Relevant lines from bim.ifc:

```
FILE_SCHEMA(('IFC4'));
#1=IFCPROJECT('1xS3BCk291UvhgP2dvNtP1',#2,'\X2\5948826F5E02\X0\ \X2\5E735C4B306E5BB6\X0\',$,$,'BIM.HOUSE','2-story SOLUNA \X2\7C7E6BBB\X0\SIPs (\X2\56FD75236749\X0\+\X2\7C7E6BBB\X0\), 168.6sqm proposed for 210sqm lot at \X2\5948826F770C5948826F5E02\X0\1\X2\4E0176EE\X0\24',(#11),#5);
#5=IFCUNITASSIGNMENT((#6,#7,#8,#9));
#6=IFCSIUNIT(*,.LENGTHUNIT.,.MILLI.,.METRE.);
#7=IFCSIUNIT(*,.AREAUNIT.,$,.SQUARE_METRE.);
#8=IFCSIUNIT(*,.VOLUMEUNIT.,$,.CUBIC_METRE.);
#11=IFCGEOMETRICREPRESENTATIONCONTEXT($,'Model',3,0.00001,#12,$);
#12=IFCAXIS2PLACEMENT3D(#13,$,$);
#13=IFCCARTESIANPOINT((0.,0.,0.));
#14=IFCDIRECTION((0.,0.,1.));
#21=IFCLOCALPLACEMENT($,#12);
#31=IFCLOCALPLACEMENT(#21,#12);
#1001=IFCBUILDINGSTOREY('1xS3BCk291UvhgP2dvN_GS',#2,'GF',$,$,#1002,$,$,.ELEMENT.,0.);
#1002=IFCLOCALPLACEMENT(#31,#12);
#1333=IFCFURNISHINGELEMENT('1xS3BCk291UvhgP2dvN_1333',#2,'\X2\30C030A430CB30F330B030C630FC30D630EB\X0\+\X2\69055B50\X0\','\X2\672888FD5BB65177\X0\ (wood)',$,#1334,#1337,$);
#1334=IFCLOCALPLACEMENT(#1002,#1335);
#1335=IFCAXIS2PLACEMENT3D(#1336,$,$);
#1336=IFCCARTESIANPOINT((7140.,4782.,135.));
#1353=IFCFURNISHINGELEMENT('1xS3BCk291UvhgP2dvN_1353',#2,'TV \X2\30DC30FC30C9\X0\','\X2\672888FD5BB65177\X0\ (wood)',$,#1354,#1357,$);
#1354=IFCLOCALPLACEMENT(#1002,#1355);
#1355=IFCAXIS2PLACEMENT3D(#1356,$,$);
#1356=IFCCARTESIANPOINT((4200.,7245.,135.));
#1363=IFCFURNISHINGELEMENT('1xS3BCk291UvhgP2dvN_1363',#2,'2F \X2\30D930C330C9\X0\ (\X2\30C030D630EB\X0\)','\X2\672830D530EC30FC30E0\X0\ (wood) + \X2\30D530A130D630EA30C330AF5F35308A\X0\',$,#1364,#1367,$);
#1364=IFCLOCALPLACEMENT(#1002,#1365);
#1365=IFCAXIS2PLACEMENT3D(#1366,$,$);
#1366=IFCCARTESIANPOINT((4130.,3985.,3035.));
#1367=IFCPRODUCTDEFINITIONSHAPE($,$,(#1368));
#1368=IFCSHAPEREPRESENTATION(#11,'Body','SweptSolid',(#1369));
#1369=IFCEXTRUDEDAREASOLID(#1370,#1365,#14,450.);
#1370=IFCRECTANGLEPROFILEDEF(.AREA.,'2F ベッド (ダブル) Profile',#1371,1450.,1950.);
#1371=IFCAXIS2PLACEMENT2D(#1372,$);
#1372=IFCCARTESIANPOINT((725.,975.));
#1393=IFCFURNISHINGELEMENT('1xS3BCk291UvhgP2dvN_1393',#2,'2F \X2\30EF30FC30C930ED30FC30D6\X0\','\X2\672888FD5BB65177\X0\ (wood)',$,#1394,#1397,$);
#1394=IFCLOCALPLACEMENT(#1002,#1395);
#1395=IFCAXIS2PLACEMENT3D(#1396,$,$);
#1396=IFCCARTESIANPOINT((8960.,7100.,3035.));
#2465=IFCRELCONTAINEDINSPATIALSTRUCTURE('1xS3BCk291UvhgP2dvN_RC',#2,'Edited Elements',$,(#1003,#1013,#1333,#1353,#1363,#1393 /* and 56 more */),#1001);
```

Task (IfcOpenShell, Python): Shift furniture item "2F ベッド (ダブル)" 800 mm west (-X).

```python
import ifcopenshell
import ifcopenshell.api.geometry
import ifcopenshell.util.placement
import ifcopenshell.util.unit

model = ifcopenshell.open("bim.ifc")
unit_scale = ifcopenshell.util.unit.calculate_unit_scale(model)

item = model.by_id(1363)
matrix = ifcopenshell.util.placement.get_local_placement(item.ObjectPlacement)
matrix[0, 3] -= 0.8 / unit_scale
ifcopenshell.api.geometry.edit_object_placement(model, product=item, matrix=matrix, is_si=False)

print(ifcopenshell.util.placement.get_local_placement(item.ObjectPlacement).round(3) + 0.0)

model.write("bim_rev.ifc")
```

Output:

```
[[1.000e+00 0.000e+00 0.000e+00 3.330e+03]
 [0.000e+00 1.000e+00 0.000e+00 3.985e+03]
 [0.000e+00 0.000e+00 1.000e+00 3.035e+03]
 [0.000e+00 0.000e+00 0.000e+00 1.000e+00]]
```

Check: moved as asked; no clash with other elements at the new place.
